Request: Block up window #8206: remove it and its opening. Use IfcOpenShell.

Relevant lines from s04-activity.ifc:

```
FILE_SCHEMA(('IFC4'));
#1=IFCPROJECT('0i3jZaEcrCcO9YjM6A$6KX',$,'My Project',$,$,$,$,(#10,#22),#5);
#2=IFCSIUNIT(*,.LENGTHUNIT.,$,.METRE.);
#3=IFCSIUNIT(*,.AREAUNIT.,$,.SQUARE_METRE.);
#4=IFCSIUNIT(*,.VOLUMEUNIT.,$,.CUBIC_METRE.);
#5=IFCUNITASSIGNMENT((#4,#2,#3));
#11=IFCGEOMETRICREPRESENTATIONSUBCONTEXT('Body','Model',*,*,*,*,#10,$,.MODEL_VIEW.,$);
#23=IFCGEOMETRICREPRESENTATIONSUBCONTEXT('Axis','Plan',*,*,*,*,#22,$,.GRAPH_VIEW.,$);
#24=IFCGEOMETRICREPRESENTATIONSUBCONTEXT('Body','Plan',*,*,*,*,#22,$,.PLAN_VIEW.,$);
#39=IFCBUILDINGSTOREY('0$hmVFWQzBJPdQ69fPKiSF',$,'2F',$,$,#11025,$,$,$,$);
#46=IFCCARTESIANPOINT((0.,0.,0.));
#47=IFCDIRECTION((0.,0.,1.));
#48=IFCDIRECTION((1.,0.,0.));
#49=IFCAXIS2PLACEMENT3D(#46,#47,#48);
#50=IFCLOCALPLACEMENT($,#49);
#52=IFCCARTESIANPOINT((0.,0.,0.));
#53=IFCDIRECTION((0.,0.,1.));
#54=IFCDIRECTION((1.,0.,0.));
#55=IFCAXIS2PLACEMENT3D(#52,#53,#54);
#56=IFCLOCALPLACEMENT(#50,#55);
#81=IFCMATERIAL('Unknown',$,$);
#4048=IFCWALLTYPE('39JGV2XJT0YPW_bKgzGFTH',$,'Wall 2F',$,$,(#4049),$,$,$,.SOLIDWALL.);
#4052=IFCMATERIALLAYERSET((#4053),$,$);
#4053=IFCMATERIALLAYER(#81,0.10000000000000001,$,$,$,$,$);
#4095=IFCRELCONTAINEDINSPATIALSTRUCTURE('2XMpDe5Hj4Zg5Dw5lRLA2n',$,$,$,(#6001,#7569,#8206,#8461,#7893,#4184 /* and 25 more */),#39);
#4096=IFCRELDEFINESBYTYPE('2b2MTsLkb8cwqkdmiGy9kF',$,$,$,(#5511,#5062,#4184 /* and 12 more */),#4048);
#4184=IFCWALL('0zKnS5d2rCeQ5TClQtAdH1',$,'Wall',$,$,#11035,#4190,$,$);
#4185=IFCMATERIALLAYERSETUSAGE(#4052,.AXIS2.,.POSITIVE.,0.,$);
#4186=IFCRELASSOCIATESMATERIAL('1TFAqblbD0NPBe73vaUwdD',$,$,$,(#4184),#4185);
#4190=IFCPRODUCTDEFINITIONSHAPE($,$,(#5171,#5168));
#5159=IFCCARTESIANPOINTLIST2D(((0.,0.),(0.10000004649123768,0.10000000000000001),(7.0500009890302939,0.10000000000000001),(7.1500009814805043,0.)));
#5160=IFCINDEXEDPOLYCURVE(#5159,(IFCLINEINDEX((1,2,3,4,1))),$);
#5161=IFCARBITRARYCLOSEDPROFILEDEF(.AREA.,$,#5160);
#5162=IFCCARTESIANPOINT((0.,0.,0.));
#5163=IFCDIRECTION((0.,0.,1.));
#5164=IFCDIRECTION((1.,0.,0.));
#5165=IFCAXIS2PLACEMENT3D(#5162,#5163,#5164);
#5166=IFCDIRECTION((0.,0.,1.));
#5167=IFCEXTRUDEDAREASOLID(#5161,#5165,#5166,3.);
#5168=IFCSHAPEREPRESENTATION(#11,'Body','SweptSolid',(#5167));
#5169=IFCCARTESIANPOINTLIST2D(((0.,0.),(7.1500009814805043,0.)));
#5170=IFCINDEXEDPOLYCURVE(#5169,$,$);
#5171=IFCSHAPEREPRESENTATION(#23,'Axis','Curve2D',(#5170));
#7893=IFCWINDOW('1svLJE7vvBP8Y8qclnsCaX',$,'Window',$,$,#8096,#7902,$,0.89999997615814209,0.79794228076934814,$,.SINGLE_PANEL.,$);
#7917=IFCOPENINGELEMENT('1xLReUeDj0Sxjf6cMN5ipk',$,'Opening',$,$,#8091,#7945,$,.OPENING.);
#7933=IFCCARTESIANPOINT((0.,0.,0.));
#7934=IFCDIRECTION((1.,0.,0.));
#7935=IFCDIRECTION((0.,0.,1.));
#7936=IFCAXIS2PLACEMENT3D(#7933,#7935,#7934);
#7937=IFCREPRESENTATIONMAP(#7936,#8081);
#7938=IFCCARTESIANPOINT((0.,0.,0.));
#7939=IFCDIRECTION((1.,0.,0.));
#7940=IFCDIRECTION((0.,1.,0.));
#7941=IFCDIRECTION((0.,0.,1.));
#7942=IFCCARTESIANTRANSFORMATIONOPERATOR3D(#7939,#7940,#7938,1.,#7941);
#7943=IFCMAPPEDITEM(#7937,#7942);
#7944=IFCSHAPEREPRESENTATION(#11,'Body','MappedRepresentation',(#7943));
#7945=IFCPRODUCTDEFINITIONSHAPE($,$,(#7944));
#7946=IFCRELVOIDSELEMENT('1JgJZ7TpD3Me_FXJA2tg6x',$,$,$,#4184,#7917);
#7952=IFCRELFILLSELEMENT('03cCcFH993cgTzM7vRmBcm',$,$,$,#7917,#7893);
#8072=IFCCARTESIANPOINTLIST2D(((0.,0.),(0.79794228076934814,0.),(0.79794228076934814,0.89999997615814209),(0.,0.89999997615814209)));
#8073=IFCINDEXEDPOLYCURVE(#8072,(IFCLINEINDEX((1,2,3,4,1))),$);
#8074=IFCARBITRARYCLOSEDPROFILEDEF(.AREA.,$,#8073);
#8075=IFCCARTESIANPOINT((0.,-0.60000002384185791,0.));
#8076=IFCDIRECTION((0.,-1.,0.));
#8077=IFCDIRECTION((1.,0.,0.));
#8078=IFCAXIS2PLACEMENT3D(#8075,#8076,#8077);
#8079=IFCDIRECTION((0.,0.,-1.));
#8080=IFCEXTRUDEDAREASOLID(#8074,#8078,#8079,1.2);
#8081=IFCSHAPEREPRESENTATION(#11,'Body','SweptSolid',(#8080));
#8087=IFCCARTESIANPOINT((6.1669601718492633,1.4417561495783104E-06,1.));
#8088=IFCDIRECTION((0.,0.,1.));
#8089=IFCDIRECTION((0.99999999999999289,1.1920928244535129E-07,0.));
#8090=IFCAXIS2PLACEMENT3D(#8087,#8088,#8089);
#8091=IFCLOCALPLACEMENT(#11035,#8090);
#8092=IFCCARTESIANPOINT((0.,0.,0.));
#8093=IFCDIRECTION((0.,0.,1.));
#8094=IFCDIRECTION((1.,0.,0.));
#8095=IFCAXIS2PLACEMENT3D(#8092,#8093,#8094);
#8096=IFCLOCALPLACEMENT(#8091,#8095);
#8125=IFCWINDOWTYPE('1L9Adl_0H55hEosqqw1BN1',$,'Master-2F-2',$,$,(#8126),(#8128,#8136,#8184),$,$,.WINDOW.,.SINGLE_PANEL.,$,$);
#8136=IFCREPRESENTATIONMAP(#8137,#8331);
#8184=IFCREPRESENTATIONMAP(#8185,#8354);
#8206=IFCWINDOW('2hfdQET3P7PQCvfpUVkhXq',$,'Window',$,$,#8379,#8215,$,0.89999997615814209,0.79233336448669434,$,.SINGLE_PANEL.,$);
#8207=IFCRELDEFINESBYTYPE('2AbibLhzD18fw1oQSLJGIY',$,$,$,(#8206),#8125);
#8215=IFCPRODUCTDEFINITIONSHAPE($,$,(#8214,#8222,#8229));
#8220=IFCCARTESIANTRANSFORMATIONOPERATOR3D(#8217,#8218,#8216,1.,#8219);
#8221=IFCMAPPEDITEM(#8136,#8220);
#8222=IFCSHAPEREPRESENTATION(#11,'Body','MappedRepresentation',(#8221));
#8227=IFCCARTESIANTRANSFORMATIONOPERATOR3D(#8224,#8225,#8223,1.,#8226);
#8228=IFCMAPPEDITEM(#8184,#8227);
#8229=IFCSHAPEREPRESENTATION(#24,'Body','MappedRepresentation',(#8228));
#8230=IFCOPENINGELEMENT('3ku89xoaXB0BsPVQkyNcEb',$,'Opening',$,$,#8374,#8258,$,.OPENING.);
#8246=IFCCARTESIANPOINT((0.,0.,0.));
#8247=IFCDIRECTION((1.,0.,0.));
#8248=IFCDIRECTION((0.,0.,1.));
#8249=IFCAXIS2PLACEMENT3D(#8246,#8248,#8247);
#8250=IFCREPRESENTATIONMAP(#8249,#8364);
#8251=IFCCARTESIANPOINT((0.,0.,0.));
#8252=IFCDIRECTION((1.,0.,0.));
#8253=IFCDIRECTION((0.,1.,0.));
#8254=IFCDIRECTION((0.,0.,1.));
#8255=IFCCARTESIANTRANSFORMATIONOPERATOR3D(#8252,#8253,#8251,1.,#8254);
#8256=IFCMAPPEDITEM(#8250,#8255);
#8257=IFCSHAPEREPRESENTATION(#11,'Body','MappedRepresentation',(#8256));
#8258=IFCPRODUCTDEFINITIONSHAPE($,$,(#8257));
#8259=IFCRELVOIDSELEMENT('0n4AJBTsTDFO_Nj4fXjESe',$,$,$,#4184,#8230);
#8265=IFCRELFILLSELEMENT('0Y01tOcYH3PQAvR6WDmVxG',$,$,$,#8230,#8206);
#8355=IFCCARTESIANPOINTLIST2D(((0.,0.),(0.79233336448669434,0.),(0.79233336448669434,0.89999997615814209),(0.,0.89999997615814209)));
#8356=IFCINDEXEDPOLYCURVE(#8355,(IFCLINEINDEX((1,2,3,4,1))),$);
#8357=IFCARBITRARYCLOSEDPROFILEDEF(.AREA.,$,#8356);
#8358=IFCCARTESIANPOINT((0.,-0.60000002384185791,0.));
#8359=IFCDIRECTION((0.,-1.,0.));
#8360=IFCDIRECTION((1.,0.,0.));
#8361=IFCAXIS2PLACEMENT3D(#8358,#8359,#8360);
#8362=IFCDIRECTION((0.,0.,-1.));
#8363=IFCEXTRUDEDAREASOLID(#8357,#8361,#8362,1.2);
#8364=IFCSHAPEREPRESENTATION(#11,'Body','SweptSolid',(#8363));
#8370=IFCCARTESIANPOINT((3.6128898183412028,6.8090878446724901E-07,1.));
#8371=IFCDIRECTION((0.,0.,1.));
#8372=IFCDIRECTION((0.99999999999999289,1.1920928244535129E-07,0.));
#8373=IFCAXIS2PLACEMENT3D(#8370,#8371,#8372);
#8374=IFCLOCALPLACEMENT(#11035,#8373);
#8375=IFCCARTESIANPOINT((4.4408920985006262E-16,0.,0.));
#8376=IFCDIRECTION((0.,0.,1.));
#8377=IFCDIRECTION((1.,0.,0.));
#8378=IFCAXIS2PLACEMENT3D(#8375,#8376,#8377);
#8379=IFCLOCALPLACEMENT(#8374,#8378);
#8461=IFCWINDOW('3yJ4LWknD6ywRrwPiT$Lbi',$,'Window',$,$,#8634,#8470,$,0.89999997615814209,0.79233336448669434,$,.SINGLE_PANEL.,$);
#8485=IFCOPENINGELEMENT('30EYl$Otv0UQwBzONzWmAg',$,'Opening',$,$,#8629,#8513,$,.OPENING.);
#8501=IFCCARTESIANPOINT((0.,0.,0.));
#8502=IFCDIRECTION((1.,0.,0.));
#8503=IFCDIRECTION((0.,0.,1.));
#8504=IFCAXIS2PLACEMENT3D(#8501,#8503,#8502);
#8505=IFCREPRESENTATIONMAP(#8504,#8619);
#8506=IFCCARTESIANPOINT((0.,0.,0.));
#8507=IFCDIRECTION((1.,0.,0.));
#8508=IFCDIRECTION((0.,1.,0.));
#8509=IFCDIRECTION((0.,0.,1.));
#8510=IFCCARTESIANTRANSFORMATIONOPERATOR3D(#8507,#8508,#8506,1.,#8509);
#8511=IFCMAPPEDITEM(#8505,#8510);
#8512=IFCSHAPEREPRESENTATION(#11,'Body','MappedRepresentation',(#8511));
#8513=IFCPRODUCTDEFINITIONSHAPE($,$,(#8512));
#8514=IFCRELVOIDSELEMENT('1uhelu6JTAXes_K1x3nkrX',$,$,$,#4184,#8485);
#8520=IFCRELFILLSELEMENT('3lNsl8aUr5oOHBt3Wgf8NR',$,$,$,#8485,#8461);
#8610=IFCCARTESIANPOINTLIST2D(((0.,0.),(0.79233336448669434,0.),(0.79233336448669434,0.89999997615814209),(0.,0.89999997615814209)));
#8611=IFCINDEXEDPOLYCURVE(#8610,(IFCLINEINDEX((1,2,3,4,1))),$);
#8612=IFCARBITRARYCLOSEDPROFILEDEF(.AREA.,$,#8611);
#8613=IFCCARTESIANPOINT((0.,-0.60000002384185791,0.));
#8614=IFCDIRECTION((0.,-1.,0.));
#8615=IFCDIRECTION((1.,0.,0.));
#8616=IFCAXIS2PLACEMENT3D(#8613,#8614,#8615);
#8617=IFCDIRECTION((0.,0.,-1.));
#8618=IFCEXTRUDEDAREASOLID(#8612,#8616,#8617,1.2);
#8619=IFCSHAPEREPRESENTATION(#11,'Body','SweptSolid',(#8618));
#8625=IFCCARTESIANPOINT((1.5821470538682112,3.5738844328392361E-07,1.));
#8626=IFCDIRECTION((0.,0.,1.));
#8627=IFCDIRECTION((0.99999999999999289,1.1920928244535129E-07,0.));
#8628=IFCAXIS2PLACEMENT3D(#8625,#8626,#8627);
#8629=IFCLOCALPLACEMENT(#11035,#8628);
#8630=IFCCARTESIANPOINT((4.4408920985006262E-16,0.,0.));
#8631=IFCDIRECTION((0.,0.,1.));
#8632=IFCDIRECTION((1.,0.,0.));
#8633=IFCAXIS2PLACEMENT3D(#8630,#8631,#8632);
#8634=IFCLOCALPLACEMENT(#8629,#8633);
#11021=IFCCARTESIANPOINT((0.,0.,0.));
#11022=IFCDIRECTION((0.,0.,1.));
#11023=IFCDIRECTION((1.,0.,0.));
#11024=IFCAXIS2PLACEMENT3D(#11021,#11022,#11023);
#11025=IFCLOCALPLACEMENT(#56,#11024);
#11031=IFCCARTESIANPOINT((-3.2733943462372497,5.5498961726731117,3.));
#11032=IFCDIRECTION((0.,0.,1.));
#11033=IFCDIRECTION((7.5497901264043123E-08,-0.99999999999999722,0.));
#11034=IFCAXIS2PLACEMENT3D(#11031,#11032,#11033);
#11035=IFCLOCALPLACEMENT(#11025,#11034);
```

```python
import ifcopenshell
import ifcopenshell.api.feature
import ifcopenshell.api.root
import ifcopenshell.geom
import ifcopenshell.util.shape

model = ifcopenshell.open("s04-activity.ifc")
settings = ifcopenshell.geom.settings()


def volume(element):
    """Net volume in cubic metres, openings subtracted."""
    shape = ifcopenshell.geom.create_shape(settings, element)
    return ifcopenshell.util.shape.get_volume(shape.geometry)


window = model.by_id(8206)
opening = window.FillsVoids[0].RelatingOpeningElement
wall = opening.VoidsElements[0].RelatingBuildingElement
before = volume(wall)

ifcopenshell.api.root.remove_product(model, product=window)
ifcopenshell.api.feature.remove_feature(model, feature=opening)

after = volume(wall)

print(f"wall volume {before:.3f} -> {after:.3f} m3")

model.write("s04-activity-out.ifc")
```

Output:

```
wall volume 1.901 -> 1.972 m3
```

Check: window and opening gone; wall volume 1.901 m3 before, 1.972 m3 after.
